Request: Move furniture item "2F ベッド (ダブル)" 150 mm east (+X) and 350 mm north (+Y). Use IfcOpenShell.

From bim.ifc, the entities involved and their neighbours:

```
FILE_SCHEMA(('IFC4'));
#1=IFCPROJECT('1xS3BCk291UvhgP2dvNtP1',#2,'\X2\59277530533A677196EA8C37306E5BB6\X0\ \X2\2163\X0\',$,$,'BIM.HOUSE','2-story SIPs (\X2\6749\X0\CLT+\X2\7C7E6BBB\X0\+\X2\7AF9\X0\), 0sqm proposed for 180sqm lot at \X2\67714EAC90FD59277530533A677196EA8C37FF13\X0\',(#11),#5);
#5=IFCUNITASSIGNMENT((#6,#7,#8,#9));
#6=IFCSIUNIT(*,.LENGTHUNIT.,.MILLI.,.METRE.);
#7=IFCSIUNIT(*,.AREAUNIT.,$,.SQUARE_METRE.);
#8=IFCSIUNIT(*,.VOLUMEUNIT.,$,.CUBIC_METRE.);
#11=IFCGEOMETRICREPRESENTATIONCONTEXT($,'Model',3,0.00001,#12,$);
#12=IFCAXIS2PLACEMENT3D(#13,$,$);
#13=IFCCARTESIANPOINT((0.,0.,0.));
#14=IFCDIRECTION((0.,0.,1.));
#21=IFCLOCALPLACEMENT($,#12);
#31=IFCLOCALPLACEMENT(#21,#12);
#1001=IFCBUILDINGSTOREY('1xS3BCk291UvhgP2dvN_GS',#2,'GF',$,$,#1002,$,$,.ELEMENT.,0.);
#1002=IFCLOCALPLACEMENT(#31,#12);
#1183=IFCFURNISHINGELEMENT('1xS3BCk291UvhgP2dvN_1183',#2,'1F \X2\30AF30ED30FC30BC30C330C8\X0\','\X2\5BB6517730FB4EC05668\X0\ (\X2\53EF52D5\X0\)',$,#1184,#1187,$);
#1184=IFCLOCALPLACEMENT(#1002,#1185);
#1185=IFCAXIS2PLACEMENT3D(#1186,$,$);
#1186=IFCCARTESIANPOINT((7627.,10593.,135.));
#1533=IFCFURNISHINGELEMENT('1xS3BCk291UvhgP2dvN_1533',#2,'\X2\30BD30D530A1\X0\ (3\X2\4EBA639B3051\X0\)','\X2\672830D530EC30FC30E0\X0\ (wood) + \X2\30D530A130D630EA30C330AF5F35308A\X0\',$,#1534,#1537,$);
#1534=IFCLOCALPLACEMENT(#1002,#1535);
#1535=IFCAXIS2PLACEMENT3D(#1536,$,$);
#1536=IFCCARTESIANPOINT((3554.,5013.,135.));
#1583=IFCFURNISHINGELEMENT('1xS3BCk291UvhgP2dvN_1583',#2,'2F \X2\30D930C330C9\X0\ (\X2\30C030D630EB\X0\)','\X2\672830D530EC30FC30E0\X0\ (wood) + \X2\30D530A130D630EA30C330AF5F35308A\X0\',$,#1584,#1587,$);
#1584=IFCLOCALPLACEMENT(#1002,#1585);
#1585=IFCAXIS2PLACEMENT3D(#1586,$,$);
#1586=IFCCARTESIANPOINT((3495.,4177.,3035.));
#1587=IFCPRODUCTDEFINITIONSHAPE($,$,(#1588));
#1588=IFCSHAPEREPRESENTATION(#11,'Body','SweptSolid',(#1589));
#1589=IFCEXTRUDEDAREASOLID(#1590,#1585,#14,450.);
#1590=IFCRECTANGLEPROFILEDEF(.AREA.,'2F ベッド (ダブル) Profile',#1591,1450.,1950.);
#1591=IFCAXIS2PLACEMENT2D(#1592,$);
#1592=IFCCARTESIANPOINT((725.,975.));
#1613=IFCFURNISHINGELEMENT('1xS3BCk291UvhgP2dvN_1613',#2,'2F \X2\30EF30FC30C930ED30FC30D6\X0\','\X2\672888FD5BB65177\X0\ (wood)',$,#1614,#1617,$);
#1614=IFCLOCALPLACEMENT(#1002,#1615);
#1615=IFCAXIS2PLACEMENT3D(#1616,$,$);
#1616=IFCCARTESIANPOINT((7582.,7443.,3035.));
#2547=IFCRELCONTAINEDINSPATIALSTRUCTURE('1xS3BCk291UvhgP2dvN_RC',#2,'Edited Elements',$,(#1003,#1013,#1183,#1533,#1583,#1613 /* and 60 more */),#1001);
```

```python
import ifcopenshell
import ifcopenshell.api.geometry
import ifcopenshell.util.placement
import ifcopenshell.util.unit

model = ifcopenshell.open("bim.ifc")
unit_scale = ifcopenshell.util.unit.calculate_unit_scale(model)

item = model.by_id(1583)
matrix = ifcopenshell.util.placement.get_local_placement(item.ObjectPlacement)
matrix[0, 3] += 0.15 / unit_scale
matrix[1, 3] += 0.35 / unit_scale
ifcopenshell.api.geometry.edit_object_placement(model, product=item, matrix=matrix, is_si=False)

print(ifcopenshell.util.placement.get_local_placement(item.ObjectPlacement).round(3) + 0.0)

model.write("bim_rev.ifc")
```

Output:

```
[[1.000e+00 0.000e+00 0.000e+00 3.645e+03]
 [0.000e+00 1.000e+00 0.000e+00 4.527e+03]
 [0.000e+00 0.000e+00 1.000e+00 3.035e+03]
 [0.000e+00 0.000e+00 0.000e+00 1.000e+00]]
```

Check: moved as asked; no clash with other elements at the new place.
